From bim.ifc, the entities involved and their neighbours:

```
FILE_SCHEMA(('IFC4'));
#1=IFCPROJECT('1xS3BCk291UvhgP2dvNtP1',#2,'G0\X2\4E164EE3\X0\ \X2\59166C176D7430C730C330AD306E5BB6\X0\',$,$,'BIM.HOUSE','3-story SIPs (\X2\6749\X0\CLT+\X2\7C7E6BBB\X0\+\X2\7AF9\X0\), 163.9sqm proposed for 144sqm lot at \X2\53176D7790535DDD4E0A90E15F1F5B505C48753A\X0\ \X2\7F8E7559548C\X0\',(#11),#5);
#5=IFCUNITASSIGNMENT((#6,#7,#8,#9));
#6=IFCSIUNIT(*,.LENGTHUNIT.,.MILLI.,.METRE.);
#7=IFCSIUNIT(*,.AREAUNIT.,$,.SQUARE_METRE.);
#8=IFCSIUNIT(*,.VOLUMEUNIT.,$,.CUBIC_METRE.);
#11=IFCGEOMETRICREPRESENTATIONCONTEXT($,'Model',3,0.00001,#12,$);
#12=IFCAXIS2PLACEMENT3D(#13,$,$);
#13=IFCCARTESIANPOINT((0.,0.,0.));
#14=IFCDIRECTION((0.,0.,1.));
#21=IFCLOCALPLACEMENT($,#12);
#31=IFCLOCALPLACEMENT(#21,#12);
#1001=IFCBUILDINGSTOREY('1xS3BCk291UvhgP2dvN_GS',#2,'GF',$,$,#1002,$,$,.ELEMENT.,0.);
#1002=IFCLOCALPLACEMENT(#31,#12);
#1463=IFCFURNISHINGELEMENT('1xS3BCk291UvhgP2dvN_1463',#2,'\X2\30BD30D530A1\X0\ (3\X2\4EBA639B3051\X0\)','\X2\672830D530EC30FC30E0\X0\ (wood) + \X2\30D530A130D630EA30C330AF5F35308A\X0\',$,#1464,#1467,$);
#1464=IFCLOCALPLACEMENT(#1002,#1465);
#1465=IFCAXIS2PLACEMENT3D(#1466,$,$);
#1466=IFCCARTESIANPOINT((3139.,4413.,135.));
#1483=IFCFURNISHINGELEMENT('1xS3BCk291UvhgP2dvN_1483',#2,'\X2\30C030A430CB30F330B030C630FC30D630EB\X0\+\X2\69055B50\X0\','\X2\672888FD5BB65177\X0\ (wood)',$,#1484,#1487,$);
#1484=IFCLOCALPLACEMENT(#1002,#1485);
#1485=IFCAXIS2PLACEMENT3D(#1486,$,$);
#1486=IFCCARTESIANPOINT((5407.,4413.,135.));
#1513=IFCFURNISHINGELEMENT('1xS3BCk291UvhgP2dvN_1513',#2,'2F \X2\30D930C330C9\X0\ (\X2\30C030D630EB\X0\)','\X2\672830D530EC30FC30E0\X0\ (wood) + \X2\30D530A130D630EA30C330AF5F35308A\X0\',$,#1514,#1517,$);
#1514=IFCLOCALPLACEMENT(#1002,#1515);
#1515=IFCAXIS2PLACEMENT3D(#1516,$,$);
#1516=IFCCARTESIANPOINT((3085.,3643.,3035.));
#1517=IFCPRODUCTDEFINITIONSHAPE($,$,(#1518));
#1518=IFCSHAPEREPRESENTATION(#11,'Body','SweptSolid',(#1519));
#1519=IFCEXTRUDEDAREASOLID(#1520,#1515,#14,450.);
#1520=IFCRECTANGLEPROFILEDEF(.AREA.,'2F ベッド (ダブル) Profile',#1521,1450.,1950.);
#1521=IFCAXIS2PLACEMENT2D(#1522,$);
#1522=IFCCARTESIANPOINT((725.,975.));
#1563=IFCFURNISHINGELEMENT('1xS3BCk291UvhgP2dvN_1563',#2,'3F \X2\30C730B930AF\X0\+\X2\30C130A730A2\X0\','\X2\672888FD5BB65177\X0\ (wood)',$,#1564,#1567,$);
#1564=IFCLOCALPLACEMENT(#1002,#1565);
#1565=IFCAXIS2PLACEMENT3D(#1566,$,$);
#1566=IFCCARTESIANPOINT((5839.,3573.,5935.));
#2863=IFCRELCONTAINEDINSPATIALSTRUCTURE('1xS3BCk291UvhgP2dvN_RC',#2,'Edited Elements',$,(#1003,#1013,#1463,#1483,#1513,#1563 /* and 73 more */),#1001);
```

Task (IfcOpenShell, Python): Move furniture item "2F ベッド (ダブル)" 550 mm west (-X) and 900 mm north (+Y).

```python
import ifcopenshell
import ifcopenshell.api.geometry
import ifcopenshell.util.placement
import ifcopenshell.util.unit

model = ifcopenshell.open("bim.ifc")
unit_scale = ifcopenshell.util.unit.calculate_unit_scale(model)

item = model.by_id(1513)
matrix = ifcopenshell.util.placement.get_local_placement(item.ObjectPlacement)
matrix[0, 3] -= 0.55 / unit_scale
matrix[1, 3] += 0.9 / unit_scale
ifcopenshell.api.geometry.edit_object_placement(model, product=item, matrix=matrix, is_si=False)

print(ifcopenshell.util.placement.get_local_placement(item.ObjectPlacement).round(3) + 0.0)

model.write("bim_v2.ifc")
```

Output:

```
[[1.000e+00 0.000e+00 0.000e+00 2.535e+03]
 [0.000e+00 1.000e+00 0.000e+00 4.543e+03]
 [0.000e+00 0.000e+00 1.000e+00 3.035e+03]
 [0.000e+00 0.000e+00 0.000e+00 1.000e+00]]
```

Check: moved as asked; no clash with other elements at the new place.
